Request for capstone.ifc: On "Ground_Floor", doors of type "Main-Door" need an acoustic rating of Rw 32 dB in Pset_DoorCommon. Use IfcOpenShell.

First a look at what the model holds.

```python
import ifcopenshell
import ifcopenshell.util.element

model = ifcopenshell.open("capstone.ifc")
print(model.schema)
storey = next(s for s in model.by_type("IfcBuildingStorey") if s.Name == "Ground_Floor")
doors = [e for e in ifcopenshell.util.element.get_decomposition(storey) if e.is_a("IfcDoor")]
seen = {}
for e in doors:
    element_type = ifcopenshell.util.element.get_type(e)
    key = (element_type.Name if element_type != e and element_type else None, ifcopenshell.util.element.get_pset(e, "Pset_DoorCommon", "AcousticRating"))
    seen[key] = seen.get(key, 0) + 1
for (name, value), count in sorted(seen.items(), key=str):
    print(count, "x", name, "|", value)
```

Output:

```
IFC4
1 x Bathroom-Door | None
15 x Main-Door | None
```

```python
import ifcopenshell
import ifcopenshell.api.pset
import ifcopenshell.util.element

model = ifcopenshell.open("capstone.ifc")

storey = next(s for s in model.by_type("IfcBuildingStorey") if s.Name == "Ground_Floor")
doors = [e for e in ifcopenshell.util.element.get_decomposition(storey) if e.is_a("IfcDoor")]

count = 0
for e in doors:
    element_type = ifcopenshell.util.element.get_type(e)
    if element_type in (None, e) or element_type.Name != "Main-Door":
        continue
    # add_pset returns the element's existing set when there is one.
    pset = ifcopenshell.api.pset.add_pset(model, product=e, name="Pset_DoorCommon")
    ifcopenshell.api.pset.edit_pset(model, pset=pset, properties={"AcousticRating": "Rw 32 dB"})
    count += 1

print(count, "doors updated")

model.write("capstone_v2.ifc")
```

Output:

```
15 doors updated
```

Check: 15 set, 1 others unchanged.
